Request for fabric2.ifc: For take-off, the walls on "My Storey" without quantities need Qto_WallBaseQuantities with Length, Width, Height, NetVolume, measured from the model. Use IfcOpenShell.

First a look at what the model holds.

```python
import ifcopenshell
import ifcopenshell.util.element
import ifcopenshell.util.unit

model = ifcopenshell.open("fabric2.ifc")
print(model.schema)
for unit_type in ("LENGTHUNIT", "AREAUNIT", "VOLUMEUNIT"):
    print(unit_type, ifcopenshell.util.unit.calculate_unit_scale(model, unit_type))
storey = next(s for s in model.by_type("IfcBuildingStorey") if s.Name == "My Storey")
walls = [e for e in ifcopenshell.util.element.get_decomposition(storey) if e.is_a("IfcWall")]
for e in sorted(walls, key=lambda e: e.id()):
    print(e.id(), e.is_a(), e.Name, list(ifcopenshell.util.element.get_psets(e, qtos_only=True)), sep=" | ")
```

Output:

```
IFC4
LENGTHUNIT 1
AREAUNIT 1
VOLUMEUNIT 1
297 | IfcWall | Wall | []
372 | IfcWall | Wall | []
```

```python
import ifcopenshell
import ifcopenshell.api.pset
import ifcopenshell.geom
import ifcopenshell.util.element
import ifcopenshell.util.shape
import ifcopenshell.util.unit

model = ifcopenshell.open("fabric2.ifc")
unit_scale = ifcopenshell.util.unit.calculate_unit_scale(model)
volume_scale = ifcopenshell.util.unit.calculate_unit_scale(model, "VOLUMEUNIT")
settings = ifcopenshell.geom.settings()

storey = next(s for s in model.by_type("IfcBuildingStorey") if s.Name == "My Storey")
walls = [e for e in ifcopenshell.util.element.get_decomposition(storey) if e.is_a("IfcWall")]

for e in sorted(walls, key=lambda e: e.id()):
    if ifcopenshell.util.element.get_psets(e, qtos_only=True, should_inherit=False):
        continue
    # Geometry comes back in metres, in the element's own axes.
    shape = ifcopenshell.geom.create_shape(settings, e)
    values = {
        "Length": ifcopenshell.util.shape.get_x(shape.geometry) / unit_scale,
        "Width": ifcopenshell.util.shape.get_y(shape.geometry) / unit_scale,
        "Height": ifcopenshell.util.shape.get_z(shape.geometry) / unit_scale,
        "NetVolume": ifcopenshell.util.shape.get_volume(shape.geometry) / volume_scale,
    }
    qto = ifcopenshell.api.pset.add_qto(model, product=e, name="Qto_WallBaseQuantities")
    ifcopenshell.api.pset.edit_qto(model, qto=qto, properties=values)
    print(e.id(), {k: round(v, 3) for k, v in values.items()})

model.write("fabric2_rev.ifc")
```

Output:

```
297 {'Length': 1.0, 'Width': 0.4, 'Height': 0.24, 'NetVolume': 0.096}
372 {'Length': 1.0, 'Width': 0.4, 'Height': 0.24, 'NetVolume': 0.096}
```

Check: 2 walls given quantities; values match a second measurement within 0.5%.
